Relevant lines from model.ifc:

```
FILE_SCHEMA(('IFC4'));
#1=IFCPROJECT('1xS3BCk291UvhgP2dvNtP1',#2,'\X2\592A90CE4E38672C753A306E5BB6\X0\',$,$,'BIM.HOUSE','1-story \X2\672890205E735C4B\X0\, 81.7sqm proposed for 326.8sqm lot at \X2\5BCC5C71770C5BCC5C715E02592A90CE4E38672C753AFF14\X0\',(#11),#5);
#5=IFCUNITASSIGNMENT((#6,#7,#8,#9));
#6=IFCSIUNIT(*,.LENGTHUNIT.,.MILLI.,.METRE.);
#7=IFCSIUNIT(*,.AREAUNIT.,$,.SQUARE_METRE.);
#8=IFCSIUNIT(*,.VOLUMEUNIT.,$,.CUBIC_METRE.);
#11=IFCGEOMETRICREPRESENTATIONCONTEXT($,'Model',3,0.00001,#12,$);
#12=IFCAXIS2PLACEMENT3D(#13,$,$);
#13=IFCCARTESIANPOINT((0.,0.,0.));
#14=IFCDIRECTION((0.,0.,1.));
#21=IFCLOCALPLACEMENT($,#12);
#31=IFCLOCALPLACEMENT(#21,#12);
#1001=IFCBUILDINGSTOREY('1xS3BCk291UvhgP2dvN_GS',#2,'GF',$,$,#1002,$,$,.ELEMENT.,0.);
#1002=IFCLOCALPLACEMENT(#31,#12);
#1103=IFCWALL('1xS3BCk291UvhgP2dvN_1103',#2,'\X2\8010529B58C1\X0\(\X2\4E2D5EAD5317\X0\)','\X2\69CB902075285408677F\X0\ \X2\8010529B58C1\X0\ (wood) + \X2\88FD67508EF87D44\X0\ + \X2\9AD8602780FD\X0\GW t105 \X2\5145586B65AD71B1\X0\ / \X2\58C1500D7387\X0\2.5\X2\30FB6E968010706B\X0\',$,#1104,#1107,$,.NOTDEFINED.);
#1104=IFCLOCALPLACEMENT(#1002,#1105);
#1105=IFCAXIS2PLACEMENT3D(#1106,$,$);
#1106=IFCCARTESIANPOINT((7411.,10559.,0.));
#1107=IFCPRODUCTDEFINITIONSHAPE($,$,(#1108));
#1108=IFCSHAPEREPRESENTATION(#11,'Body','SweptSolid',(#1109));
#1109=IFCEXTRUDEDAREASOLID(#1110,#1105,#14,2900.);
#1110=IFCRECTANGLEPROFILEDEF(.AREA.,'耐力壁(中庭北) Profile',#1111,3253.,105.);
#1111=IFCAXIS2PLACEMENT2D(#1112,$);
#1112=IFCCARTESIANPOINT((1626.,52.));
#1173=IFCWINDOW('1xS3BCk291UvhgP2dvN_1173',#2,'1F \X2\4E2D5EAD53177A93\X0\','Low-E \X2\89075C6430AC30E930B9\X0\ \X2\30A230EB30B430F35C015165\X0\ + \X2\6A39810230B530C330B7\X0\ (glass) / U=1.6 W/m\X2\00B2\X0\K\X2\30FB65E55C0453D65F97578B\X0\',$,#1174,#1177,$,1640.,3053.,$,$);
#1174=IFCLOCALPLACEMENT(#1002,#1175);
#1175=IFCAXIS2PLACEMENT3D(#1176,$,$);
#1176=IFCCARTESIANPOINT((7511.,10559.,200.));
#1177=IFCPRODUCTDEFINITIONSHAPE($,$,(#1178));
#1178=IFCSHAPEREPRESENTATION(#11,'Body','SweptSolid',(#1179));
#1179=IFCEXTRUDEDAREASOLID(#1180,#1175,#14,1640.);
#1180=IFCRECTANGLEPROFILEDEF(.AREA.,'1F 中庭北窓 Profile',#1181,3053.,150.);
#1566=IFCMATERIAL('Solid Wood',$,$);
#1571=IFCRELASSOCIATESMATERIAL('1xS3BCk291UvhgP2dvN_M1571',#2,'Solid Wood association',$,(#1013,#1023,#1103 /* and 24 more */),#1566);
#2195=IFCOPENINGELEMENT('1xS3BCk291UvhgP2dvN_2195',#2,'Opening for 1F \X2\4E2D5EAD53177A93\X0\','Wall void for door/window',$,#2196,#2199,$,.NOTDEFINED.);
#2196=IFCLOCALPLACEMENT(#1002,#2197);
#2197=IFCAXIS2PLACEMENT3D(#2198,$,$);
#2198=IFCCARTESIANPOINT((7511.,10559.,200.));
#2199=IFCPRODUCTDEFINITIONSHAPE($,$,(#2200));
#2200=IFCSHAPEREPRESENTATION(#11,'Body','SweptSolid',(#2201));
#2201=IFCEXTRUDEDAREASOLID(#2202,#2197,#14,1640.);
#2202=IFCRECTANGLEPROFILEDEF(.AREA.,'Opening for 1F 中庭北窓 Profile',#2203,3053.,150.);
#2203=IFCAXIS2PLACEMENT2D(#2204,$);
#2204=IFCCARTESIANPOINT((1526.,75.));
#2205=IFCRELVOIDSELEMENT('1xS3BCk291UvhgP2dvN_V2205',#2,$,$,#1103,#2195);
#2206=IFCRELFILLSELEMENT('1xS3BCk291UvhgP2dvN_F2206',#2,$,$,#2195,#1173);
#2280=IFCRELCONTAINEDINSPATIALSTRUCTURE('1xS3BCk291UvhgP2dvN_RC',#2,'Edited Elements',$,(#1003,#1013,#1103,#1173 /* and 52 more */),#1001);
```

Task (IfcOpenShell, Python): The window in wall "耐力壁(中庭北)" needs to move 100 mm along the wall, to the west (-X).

```python
import ifcopenshell
import ifcopenshell.api.geometry
import ifcopenshell.util.placement

model = ifcopenshell.open("model.ifc")

window = model.by_guid("1xS3BCk291UvhgP2dvN_1173")
opening = window.FillsVoids[0].RelatingOpeningElement
wall = opening.VoidsElements[0].RelatingBuildingElement

wall_matrix = ifcopenshell.util.placement.get_local_placement(wall.ObjectPlacement)
shift = wall_matrix[:3, 0] * -100.0
before = ifcopenshell.util.placement.get_local_placement(window.ObjectPlacement)[:3, 3].copy()

# The window is not placed relative to its opening, so move both.
for product in (opening, window):
    matrix = ifcopenshell.util.placement.get_local_placement(product.ObjectPlacement)
    matrix[:3, 3] += shift
    ifcopenshell.api.geometry.edit_object_placement(model, product=product, matrix=matrix, is_si=False)

after = ifcopenshell.util.placement.get_local_placement(window.ObjectPlacement)[:3, 3]
print("window moved by", (after - before).round(3) + 0.0)

model.write("model_edited.ifc")
```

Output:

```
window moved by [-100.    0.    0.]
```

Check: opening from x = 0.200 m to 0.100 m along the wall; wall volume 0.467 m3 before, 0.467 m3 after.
